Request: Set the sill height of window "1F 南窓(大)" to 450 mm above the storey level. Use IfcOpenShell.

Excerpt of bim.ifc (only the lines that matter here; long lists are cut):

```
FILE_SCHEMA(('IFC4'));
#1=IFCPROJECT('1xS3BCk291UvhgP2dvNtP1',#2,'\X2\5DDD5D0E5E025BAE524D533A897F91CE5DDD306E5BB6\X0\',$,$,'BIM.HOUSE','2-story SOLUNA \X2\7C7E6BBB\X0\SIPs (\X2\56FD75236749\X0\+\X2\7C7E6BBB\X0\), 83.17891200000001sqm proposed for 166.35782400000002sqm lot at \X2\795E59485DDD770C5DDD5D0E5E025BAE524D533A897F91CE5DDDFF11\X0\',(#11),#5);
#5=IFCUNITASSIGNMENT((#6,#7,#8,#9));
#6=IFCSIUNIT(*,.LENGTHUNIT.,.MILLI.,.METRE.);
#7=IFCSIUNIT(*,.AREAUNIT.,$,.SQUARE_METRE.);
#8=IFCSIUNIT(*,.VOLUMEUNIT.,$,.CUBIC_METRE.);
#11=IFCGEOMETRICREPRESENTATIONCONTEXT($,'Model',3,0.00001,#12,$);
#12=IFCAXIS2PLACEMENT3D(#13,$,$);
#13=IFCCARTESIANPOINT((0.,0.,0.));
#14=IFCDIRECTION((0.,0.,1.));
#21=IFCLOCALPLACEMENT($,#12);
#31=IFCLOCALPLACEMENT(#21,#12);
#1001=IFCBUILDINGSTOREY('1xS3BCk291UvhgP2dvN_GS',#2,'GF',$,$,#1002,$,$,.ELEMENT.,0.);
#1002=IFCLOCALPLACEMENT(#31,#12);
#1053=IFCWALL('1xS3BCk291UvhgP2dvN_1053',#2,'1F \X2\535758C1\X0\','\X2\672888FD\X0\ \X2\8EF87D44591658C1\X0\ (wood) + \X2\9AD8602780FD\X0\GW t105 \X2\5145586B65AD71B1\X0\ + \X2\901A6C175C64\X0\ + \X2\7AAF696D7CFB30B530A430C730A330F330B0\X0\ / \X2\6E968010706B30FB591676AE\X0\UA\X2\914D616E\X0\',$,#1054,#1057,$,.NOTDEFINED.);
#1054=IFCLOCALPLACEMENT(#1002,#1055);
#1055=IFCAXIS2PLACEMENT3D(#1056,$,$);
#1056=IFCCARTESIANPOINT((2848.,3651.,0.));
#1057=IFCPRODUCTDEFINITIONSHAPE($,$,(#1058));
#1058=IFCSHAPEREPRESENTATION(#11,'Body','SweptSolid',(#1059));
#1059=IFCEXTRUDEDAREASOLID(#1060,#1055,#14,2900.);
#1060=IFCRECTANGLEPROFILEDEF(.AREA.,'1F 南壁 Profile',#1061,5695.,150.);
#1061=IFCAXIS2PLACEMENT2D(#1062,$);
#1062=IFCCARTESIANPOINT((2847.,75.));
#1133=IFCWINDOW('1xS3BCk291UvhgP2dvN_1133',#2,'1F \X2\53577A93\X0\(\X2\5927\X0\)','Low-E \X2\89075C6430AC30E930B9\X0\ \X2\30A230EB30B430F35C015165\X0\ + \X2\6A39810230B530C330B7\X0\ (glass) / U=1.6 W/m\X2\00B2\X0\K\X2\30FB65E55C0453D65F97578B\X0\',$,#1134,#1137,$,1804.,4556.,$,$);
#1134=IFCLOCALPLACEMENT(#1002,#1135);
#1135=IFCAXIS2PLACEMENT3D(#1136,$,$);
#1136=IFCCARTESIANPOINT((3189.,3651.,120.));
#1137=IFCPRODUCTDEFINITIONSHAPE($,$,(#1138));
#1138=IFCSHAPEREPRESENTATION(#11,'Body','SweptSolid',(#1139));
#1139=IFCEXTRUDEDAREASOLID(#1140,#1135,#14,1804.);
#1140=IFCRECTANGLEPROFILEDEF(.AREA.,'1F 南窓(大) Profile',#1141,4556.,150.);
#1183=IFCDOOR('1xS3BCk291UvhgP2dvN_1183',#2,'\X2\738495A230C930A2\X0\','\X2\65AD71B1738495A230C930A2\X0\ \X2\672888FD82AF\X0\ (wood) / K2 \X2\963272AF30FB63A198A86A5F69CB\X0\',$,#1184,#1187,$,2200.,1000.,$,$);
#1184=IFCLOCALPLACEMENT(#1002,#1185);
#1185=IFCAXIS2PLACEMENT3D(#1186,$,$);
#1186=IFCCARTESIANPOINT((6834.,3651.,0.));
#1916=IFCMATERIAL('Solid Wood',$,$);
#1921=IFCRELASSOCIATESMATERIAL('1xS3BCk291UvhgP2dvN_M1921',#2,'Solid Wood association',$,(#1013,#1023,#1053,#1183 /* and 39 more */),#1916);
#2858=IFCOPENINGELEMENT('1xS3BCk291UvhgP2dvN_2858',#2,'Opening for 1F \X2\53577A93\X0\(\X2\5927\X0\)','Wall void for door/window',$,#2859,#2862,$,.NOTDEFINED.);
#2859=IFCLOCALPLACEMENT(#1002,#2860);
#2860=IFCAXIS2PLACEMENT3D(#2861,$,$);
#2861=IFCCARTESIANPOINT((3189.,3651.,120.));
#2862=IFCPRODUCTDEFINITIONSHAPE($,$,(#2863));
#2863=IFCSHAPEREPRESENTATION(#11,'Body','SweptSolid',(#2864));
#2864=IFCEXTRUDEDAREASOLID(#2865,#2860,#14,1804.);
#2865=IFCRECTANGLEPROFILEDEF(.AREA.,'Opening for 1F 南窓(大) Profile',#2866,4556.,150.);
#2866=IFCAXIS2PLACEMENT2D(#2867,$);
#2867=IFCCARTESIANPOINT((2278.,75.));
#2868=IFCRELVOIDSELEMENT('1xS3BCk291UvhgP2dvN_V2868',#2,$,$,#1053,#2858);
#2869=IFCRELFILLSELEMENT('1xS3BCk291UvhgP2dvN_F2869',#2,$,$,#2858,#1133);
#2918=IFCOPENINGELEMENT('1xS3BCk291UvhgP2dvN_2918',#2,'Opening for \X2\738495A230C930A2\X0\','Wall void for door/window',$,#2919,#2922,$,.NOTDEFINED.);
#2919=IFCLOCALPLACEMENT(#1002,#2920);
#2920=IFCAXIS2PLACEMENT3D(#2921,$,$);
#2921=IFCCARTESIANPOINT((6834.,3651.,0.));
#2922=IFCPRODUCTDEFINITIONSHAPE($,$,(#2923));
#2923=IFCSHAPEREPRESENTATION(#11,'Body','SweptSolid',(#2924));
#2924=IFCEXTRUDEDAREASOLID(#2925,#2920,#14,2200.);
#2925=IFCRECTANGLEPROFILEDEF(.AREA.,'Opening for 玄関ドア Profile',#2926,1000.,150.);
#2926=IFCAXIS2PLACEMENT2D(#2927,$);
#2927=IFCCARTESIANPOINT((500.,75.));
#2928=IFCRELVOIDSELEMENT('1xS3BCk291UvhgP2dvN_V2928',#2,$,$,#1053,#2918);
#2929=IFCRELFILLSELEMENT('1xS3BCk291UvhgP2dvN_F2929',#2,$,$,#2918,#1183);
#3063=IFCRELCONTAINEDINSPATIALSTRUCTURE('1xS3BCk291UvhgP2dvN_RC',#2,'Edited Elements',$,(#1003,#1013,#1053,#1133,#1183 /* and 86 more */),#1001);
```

```python
import numpy as np
import ifcopenshell
import ifcopenshell.api.geometry
import ifcopenshell.geom
import ifcopenshell.util.element
import ifcopenshell.util.placement
import ifcopenshell.util.shape
import ifcopenshell.util.unit

model = ifcopenshell.open("bim.ifc")
unit_scale = ifcopenshell.util.unit.calculate_unit_scale(model)

window = model.by_id(1133)
opening = window.FillsVoids[0].RelatingOpeningElement
storey = ifcopenshell.util.element.get_container(window, ifc_class="IfcBuildingStorey")
level = ifcopenshell.util.placement.get_local_placement(storey.ObjectPlacement)[2, 3]

# The opening's origin need not be at the sill, so measure its lowest point.
shape = ifcopenshell.geom.create_shape(ifcopenshell.geom.settings(), opening)
bottom = ifcopenshell.util.shape.get_shape_bottom_elevation(shape, shape.geometry) / unit_scale
dz = level + 0.45 / unit_scale - bottom

shift = np.array([0.0, 0.0, dz])
# The window is not placed relative to its opening, so move both.
for product in (opening, window):
    matrix = ifcopenshell.util.placement.get_local_placement(product.ObjectPlacement)
    matrix[:3, 3] += shift
    ifcopenshell.api.geometry.edit_object_placement(model, product=product, matrix=matrix, is_si=False)

print(f"moved by {dz * unit_scale:+.3f} m")

model.write("bim_updated.ifc")
```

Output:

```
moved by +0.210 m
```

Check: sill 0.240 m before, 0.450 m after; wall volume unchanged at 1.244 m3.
